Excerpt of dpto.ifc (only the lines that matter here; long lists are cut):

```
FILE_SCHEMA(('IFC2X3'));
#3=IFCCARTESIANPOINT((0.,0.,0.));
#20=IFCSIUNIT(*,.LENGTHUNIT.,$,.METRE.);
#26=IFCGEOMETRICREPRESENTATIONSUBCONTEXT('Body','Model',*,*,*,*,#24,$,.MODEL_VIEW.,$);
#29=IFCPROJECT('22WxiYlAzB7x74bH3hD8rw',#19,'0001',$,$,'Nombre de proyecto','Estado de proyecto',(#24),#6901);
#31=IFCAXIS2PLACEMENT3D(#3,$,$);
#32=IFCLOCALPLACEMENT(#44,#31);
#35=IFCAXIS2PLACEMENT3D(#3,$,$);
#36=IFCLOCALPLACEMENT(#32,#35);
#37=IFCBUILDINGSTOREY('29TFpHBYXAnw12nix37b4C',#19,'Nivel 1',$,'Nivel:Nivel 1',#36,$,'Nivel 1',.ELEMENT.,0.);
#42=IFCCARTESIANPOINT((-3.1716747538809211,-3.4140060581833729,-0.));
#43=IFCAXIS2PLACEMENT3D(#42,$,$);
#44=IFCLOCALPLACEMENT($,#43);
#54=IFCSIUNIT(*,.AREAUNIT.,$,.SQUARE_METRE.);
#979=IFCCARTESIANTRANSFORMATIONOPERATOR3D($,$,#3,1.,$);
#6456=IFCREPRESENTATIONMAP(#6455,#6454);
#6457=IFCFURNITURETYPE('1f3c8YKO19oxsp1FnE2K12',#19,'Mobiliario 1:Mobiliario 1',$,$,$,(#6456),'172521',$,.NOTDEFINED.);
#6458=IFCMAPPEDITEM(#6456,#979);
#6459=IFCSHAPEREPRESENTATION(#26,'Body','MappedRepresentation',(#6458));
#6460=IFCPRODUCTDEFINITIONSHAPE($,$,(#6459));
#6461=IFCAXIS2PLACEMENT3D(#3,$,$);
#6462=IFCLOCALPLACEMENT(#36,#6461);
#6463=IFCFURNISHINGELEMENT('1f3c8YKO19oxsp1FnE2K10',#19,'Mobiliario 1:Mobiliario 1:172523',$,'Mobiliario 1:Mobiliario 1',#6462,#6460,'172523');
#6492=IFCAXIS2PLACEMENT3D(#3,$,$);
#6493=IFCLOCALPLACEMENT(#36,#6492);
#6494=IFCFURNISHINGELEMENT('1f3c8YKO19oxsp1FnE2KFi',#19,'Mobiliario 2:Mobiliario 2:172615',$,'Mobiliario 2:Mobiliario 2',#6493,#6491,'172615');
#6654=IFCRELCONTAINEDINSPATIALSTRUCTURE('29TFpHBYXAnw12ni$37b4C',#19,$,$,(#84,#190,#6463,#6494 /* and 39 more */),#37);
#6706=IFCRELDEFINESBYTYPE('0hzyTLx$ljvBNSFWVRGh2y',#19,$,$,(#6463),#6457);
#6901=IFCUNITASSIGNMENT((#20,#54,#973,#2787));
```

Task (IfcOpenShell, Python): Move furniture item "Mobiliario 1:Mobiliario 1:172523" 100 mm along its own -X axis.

```python
import ifcopenshell
import ifcopenshell.api.geometry
import ifcopenshell.util.placement

model = ifcopenshell.open("dpto.ifc")

item = model.by_id(6463)
matrix = ifcopenshell.util.placement.get_local_placement(item.ObjectPlacement)
matrix[:3, 3] -= matrix[:3, 0] * 0.1
ifcopenshell.api.geometry.edit_object_placement(model, product=item, matrix=matrix, is_si=False)

print(ifcopenshell.util.placement.get_local_placement(item.ObjectPlacement).round(3) + 0.0)

model.write("dpto_rev.ifc")
```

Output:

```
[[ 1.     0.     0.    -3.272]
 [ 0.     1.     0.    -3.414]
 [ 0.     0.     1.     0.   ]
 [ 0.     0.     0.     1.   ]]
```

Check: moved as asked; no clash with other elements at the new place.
